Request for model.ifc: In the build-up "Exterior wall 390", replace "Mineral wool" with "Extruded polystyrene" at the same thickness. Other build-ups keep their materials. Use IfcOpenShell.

First a look at what the model holds.

```python
import ifcopenshell
import ifcopenshell.util.element

model = ifcopenshell.open("model.ifc")
print(model.schema)
for layer_set in model.by_type("IfcMaterialLayerSet"):
    if layer_set.LayerSetName == "Exterior wall 390":
        for layer in layer_set.MaterialLayers:
            print(layer.id(), layer.Material and layer.Material.Name, layer.LayerThickness, sep=" | ")
        print(len(ifcopenshell.util.element.get_elements_by_material(model, layer_set)), "elements and types use it")
print(sorted(m.Name for m in model.by_type("IfcMaterial") if m.Name)[:60])
```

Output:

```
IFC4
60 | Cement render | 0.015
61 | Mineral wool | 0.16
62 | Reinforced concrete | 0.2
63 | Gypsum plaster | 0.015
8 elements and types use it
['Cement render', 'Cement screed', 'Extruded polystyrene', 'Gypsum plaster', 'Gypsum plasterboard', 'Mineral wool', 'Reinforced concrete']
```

```python
import ifcopenshell
import ifcopenshell.api.material

model = ifcopenshell.open("model.ifc")

layer_set = next(s for s in model.by_type("IfcMaterialLayerSet") if s.LayerSetName == "Exterior wall 390")
layer = next(l for l in layer_set.MaterialLayers if l.Material and l.Material.Name == "Mineral wool")
material = next(m for m in model.by_type("IfcMaterial") if m.Name == "Extruded polystyrene")

# Point this one layer at the other material; renaming the old one would change it everywhere.
ifcopenshell.api.material.edit_layer(model, layer=layer, attributes={"Name": material.Name}, material=material)

print([l.Material.Name if l.Material else None for l in layer_set.MaterialLayers])

model.write("model_updated.ifc")
```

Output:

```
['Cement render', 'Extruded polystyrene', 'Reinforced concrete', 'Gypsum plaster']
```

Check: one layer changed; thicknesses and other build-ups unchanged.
